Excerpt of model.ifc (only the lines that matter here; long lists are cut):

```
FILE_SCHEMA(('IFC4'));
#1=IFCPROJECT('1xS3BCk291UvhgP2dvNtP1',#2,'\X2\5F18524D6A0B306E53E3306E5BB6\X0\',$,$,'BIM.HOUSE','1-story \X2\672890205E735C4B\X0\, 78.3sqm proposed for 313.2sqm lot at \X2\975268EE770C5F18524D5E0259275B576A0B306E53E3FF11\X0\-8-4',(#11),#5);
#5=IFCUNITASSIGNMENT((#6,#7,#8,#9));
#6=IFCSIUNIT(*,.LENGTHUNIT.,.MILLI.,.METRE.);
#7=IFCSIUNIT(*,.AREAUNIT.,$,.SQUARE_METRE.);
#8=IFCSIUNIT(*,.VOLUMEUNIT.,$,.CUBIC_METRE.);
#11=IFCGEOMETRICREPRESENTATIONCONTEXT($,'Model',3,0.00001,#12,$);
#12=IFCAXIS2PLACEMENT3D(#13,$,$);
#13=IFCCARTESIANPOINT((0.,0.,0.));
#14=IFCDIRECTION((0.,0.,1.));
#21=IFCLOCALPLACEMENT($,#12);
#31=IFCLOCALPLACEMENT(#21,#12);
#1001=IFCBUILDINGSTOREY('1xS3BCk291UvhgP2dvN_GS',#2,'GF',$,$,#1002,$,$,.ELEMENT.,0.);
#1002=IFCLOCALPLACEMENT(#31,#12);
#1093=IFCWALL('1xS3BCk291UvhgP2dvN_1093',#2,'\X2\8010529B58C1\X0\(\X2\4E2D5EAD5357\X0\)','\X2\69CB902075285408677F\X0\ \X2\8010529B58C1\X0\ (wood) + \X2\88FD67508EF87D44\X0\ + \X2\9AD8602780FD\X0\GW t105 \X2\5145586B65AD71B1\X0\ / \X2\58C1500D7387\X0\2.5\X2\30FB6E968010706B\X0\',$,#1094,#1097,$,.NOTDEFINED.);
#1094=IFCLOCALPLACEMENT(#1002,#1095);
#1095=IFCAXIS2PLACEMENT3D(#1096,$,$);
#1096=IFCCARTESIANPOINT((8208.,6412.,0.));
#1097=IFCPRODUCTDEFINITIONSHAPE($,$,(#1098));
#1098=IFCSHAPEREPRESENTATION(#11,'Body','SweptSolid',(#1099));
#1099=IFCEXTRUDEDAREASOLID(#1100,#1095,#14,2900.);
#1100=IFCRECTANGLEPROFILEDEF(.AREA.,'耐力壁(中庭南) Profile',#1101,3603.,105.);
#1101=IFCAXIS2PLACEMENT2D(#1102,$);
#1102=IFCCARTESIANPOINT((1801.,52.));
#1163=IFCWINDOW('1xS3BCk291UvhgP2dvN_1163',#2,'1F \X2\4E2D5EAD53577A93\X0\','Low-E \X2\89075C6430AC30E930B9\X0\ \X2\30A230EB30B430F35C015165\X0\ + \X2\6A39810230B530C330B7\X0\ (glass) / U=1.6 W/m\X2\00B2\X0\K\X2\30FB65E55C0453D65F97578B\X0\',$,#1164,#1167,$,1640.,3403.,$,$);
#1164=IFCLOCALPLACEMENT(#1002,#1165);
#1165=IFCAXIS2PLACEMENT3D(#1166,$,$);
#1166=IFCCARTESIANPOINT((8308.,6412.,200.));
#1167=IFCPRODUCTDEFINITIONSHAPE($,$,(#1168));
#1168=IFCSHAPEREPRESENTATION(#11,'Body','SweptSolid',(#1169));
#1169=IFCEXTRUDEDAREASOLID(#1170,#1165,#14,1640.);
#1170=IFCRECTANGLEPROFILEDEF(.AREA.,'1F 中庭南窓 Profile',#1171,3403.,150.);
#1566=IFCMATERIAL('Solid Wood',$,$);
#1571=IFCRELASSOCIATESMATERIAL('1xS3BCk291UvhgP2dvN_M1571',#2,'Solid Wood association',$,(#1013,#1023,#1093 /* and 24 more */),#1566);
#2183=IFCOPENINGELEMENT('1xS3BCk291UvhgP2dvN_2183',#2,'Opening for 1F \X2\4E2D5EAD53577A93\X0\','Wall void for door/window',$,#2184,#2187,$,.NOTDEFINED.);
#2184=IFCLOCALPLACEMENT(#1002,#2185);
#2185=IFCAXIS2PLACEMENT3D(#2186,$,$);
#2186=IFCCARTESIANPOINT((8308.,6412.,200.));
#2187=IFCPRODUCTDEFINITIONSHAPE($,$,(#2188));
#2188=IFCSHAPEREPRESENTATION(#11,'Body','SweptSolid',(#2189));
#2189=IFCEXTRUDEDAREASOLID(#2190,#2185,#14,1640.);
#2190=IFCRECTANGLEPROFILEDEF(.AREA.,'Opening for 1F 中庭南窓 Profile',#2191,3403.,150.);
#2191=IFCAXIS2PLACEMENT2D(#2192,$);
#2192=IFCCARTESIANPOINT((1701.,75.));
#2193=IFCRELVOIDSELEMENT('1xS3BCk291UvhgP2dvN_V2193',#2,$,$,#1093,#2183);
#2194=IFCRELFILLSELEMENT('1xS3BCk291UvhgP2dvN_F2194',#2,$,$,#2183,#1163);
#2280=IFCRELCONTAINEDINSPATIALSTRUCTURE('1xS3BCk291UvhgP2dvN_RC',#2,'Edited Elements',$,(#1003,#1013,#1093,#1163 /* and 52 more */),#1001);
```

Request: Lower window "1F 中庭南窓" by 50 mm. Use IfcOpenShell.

```python
import numpy as np
import ifcopenshell
import ifcopenshell.api.geometry
import ifcopenshell.util.placement
import ifcopenshell.util.unit

model = ifcopenshell.open("model.ifc")
unit_scale = ifcopenshell.util.unit.calculate_unit_scale(model)

window = model.by_guid("1xS3BCk291UvhgP2dvN_1163")
opening = window.FillsVoids[0].RelatingOpeningElement
dz = -50.0

shift = np.array([0.0, 0.0, dz])
# The window is not placed relative to its opening, so move both.
for product in (opening, window):
    matrix = ifcopenshell.util.placement.get_local_placement(product.ObjectPlacement)
    matrix[:3, 3] += shift
    ifcopenshell.api.geometry.edit_object_placement(model, product=product, matrix=matrix, is_si=False)

print(f"moved by {dz * unit_scale:+.3f} m")

model.write("model-out.ifc")
```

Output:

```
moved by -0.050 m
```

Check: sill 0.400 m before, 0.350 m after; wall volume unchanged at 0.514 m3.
